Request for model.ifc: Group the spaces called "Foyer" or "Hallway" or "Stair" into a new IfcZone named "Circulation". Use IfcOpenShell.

First a look at what the model holds.

```python
import ifcopenshell

model = ifcopenshell.open("model.ifc")
print(model.schema)
seen = {}
for space in model.by_type("IfcSpace"):
    seen[space.LongName] = seen.get(space.LongName, 0) + 1
for name, count in sorted(seen.items(), key=str):
    print(count, "x", name)
print("zones:", [z.Name for z in model.by_type("IfcZone")][:20])
```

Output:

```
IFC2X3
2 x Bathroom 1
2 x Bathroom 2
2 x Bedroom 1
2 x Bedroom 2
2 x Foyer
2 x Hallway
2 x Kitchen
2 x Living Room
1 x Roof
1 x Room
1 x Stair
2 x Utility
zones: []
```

```python
import ifcopenshell
import ifcopenshell.api.group
import ifcopenshell.api.root

model = ifcopenshell.open("model.ifc")

names = {"Foyer", "Hallway", "Stair"}
spaces = [s for s in model.by_type("IfcSpace") if s.LongName in names]

zone = ifcopenshell.api.root.create_entity(model, ifc_class="IfcZone", name="Circulation")
ifcopenshell.api.group.assign_group(model, products=spaces, group=zone)
print(len(spaces), "spaces in", zone.Name)

model.write("model_edited.ifc")
```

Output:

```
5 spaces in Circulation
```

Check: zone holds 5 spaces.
